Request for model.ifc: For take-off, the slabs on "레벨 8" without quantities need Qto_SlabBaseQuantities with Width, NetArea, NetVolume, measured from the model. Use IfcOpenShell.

First a look at what the model holds.

```python
import ifcopenshell
import ifcopenshell.util.element
import ifcopenshell.util.unit

model = ifcopenshell.open("model.ifc")
print(model.schema)
for unit_type in ("LENGTHUNIT", "AREAUNIT", "VOLUMEUNIT"):
    print(unit_type, ifcopenshell.util.unit.calculate_unit_scale(model, unit_type))
storey = next(s for s in model.by_type("IfcBuildingStorey") if s.Name == "레벨 8")
slabs = [e for e in ifcopenshell.util.element.get_decomposition(storey) if e.is_a("IfcSlab")]
for e in sorted(slabs, key=lambda e: e.id()):
    print(e.id(), e.is_a(), e.Name, list(ifcopenshell.util.element.get_psets(e, qtos_only=True)), sep=" | ")
```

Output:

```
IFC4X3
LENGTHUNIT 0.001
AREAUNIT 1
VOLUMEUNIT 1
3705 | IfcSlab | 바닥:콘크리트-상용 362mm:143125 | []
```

```python
import ifcopenshell
import ifcopenshell.api.pset
import ifcopenshell.geom
import ifcopenshell.util.element
import ifcopenshell.util.shape
import ifcopenshell.util.unit

model = ifcopenshell.open("model.ifc")
unit_scale = ifcopenshell.util.unit.calculate_unit_scale(model)
area_scale = ifcopenshell.util.unit.calculate_unit_scale(model, "AREAUNIT")
volume_scale = ifcopenshell.util.unit.calculate_unit_scale(model, "VOLUMEUNIT")
settings = ifcopenshell.geom.settings()

storey = next(s for s in model.by_type("IfcBuildingStorey") if s.Name == "레벨 8")
slabs = [e for e in ifcopenshell.util.element.get_decomposition(storey) if e.is_a("IfcSlab")]

for e in sorted(slabs, key=lambda e: e.id()):
    if ifcopenshell.util.element.get_psets(e, qtos_only=True, should_inherit=False):
        continue
    # Geometry comes back in metres, in the element's own axes.
    shape = ifcopenshell.geom.create_shape(settings, e)
    values = {
        "Width": ifcopenshell.util.shape.get_z(shape.geometry) / unit_scale,
        "NetArea": ifcopenshell.util.shape.get_footprint_area(shape.geometry) / area_scale,
        "NetVolume": ifcopenshell.util.shape.get_volume(shape.geometry) / volume_scale,
    }
    qto = ifcopenshell.api.pset.add_qto(model, product=e, name="Qto_SlabBaseQuantities")
    ifcopenshell.api.pset.edit_qto(model, qto=qto, properties=values)
    print(e.id(), {k: round(v, 3) for k, v in values.items()})

model.write("model-out.ifc")
```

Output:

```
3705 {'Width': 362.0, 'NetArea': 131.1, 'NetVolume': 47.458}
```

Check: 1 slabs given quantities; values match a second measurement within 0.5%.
